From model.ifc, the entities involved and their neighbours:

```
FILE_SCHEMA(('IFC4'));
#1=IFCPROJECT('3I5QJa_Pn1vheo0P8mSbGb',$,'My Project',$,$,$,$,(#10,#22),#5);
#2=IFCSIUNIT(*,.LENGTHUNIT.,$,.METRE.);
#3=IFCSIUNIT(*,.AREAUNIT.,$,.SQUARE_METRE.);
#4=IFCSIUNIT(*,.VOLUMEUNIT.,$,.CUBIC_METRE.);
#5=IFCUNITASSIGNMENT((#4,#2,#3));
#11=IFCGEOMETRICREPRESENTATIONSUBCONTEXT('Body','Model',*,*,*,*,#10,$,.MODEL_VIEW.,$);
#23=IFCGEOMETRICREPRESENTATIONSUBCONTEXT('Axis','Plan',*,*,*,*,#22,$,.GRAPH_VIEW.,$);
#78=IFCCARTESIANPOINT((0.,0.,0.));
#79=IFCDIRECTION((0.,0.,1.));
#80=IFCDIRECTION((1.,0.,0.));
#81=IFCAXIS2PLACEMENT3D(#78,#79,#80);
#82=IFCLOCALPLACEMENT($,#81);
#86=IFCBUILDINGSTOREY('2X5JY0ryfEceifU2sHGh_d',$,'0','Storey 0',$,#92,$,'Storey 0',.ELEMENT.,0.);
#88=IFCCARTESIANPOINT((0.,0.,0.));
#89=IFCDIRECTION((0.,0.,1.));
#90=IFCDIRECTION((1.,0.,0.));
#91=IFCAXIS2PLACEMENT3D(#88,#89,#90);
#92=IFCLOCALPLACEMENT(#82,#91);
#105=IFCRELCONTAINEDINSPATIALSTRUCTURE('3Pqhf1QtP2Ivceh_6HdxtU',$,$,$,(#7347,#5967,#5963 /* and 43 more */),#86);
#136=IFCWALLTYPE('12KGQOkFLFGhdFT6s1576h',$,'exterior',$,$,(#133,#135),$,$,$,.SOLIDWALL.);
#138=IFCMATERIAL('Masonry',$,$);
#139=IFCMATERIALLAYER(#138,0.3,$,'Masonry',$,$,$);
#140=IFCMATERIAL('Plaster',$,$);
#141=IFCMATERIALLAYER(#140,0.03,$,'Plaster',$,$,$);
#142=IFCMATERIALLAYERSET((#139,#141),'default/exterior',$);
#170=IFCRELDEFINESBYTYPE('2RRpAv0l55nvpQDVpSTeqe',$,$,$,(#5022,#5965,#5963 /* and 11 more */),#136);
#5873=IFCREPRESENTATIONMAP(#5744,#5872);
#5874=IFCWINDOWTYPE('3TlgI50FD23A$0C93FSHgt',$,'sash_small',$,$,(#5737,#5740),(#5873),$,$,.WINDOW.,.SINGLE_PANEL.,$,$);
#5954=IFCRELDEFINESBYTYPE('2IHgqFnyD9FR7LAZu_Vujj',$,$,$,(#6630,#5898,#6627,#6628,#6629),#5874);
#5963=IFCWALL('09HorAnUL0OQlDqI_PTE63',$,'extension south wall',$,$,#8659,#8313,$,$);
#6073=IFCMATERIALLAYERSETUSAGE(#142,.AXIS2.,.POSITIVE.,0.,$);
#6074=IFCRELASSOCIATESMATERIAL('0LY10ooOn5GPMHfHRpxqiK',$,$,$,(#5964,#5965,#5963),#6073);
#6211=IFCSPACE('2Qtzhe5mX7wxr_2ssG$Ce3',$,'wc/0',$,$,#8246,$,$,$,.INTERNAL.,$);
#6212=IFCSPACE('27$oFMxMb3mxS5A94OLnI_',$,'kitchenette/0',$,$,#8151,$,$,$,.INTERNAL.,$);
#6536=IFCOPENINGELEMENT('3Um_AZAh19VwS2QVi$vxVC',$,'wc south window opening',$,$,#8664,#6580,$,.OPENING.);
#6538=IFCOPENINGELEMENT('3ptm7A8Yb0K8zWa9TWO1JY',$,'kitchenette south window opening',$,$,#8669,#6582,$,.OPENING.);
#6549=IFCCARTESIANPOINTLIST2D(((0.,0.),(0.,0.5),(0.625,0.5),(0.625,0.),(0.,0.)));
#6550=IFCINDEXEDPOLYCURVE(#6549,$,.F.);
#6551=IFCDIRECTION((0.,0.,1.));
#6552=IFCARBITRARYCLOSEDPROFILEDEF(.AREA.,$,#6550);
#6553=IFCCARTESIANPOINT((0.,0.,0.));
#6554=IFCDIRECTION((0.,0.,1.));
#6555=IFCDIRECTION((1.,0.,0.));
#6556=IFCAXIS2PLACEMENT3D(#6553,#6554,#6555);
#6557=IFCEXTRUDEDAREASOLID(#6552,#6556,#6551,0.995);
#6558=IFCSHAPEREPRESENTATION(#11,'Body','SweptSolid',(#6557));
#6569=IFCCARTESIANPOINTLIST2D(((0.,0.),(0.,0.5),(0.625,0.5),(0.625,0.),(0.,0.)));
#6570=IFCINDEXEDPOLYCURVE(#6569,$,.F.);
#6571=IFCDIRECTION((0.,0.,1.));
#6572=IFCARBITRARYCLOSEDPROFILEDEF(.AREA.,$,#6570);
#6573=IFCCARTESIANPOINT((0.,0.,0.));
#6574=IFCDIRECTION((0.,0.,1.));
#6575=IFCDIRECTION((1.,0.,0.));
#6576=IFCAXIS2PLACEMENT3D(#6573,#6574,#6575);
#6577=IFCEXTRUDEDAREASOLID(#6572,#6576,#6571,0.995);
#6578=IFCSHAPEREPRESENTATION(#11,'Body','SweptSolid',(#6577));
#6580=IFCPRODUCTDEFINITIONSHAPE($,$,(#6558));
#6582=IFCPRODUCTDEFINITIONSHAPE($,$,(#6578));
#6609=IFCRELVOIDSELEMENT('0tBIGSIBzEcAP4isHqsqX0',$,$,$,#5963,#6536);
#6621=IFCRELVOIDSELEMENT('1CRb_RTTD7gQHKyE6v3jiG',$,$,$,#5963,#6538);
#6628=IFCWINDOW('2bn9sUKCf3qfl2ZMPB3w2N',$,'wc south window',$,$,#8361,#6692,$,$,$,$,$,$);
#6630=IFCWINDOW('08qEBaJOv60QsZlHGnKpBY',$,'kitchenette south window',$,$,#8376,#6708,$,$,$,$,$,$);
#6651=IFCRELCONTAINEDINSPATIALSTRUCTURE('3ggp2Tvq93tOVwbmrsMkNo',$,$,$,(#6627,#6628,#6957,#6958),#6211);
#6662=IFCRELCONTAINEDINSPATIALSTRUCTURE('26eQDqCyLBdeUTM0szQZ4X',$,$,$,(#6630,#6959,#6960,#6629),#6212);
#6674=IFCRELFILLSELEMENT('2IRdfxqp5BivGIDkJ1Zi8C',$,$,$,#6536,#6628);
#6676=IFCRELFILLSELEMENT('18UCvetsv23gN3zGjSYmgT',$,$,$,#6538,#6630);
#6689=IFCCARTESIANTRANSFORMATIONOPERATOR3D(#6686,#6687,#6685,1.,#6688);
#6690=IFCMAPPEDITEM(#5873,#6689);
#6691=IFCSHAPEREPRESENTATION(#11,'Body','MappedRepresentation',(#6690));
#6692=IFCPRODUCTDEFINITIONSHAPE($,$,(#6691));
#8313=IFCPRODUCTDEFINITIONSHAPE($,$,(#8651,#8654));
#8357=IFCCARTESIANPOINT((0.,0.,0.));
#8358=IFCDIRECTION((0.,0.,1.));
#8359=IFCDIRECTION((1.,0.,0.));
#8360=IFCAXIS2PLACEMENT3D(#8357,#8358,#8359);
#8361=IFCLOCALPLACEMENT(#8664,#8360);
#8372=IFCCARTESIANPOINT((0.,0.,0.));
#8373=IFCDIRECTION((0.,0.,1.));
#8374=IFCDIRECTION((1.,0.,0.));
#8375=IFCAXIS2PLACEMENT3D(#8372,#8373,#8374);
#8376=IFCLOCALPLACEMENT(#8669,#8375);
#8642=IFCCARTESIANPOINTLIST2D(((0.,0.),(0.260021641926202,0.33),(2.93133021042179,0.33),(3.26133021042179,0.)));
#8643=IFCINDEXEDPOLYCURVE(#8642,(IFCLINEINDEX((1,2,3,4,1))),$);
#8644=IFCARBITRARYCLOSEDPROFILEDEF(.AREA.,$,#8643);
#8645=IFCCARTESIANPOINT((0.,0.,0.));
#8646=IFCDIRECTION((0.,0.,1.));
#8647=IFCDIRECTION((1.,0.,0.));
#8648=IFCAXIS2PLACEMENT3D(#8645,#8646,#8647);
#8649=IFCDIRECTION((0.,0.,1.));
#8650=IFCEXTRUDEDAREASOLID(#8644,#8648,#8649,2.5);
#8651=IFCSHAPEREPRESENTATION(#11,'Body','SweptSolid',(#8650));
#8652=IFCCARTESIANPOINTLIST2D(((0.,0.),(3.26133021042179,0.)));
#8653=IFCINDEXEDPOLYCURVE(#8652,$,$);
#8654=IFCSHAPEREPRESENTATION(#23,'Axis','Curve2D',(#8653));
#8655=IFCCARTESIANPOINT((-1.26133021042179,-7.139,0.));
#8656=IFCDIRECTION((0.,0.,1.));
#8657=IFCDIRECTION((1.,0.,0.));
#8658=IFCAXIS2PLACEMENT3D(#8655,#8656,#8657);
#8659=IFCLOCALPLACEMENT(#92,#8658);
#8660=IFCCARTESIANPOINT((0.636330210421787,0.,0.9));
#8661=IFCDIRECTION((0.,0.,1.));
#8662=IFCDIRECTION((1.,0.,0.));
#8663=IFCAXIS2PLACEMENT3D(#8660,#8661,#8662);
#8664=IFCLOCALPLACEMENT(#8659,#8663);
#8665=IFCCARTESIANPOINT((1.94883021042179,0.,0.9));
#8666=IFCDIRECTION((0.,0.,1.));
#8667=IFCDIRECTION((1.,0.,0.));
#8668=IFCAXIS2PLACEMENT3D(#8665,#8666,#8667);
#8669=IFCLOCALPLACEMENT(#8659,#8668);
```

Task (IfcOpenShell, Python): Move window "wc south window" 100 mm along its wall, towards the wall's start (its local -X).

```python
import ifcopenshell
import ifcopenshell.api.geometry
import ifcopenshell.util.placement
import ifcopenshell.util.unit

model = ifcopenshell.open("model.ifc")
unit_scale = ifcopenshell.util.unit.calculate_unit_scale(model)

window = model.by_id(6628)
opening = window.FillsVoids[0].RelatingOpeningElement
wall = opening.VoidsElements[0].RelatingBuildingElement

wall_matrix = ifcopenshell.util.placement.get_local_placement(wall.ObjectPlacement)
shift = wall_matrix[:3, 0] * -0.1 / unit_scale
before = ifcopenshell.util.placement.get_local_placement(window.ObjectPlacement)[:3, 3].copy()

# The window is placed relative to its opening, so it follows when the opening moves.
matrix = ifcopenshell.util.placement.get_local_placement(opening.ObjectPlacement)
matrix[:3, 3] += shift
ifcopenshell.api.geometry.edit_object_placement(
    model, product=opening, matrix=matrix, is_si=False, should_transform_children=True
)

after = ifcopenshell.util.placement.get_local_placement(window.ObjectPlacement)[:3, 3]
print("window moved by", (after - before).round(3) + 0.0)

model.write("model-out.ifc")
```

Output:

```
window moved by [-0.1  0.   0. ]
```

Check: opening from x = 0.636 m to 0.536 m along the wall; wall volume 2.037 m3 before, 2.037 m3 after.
